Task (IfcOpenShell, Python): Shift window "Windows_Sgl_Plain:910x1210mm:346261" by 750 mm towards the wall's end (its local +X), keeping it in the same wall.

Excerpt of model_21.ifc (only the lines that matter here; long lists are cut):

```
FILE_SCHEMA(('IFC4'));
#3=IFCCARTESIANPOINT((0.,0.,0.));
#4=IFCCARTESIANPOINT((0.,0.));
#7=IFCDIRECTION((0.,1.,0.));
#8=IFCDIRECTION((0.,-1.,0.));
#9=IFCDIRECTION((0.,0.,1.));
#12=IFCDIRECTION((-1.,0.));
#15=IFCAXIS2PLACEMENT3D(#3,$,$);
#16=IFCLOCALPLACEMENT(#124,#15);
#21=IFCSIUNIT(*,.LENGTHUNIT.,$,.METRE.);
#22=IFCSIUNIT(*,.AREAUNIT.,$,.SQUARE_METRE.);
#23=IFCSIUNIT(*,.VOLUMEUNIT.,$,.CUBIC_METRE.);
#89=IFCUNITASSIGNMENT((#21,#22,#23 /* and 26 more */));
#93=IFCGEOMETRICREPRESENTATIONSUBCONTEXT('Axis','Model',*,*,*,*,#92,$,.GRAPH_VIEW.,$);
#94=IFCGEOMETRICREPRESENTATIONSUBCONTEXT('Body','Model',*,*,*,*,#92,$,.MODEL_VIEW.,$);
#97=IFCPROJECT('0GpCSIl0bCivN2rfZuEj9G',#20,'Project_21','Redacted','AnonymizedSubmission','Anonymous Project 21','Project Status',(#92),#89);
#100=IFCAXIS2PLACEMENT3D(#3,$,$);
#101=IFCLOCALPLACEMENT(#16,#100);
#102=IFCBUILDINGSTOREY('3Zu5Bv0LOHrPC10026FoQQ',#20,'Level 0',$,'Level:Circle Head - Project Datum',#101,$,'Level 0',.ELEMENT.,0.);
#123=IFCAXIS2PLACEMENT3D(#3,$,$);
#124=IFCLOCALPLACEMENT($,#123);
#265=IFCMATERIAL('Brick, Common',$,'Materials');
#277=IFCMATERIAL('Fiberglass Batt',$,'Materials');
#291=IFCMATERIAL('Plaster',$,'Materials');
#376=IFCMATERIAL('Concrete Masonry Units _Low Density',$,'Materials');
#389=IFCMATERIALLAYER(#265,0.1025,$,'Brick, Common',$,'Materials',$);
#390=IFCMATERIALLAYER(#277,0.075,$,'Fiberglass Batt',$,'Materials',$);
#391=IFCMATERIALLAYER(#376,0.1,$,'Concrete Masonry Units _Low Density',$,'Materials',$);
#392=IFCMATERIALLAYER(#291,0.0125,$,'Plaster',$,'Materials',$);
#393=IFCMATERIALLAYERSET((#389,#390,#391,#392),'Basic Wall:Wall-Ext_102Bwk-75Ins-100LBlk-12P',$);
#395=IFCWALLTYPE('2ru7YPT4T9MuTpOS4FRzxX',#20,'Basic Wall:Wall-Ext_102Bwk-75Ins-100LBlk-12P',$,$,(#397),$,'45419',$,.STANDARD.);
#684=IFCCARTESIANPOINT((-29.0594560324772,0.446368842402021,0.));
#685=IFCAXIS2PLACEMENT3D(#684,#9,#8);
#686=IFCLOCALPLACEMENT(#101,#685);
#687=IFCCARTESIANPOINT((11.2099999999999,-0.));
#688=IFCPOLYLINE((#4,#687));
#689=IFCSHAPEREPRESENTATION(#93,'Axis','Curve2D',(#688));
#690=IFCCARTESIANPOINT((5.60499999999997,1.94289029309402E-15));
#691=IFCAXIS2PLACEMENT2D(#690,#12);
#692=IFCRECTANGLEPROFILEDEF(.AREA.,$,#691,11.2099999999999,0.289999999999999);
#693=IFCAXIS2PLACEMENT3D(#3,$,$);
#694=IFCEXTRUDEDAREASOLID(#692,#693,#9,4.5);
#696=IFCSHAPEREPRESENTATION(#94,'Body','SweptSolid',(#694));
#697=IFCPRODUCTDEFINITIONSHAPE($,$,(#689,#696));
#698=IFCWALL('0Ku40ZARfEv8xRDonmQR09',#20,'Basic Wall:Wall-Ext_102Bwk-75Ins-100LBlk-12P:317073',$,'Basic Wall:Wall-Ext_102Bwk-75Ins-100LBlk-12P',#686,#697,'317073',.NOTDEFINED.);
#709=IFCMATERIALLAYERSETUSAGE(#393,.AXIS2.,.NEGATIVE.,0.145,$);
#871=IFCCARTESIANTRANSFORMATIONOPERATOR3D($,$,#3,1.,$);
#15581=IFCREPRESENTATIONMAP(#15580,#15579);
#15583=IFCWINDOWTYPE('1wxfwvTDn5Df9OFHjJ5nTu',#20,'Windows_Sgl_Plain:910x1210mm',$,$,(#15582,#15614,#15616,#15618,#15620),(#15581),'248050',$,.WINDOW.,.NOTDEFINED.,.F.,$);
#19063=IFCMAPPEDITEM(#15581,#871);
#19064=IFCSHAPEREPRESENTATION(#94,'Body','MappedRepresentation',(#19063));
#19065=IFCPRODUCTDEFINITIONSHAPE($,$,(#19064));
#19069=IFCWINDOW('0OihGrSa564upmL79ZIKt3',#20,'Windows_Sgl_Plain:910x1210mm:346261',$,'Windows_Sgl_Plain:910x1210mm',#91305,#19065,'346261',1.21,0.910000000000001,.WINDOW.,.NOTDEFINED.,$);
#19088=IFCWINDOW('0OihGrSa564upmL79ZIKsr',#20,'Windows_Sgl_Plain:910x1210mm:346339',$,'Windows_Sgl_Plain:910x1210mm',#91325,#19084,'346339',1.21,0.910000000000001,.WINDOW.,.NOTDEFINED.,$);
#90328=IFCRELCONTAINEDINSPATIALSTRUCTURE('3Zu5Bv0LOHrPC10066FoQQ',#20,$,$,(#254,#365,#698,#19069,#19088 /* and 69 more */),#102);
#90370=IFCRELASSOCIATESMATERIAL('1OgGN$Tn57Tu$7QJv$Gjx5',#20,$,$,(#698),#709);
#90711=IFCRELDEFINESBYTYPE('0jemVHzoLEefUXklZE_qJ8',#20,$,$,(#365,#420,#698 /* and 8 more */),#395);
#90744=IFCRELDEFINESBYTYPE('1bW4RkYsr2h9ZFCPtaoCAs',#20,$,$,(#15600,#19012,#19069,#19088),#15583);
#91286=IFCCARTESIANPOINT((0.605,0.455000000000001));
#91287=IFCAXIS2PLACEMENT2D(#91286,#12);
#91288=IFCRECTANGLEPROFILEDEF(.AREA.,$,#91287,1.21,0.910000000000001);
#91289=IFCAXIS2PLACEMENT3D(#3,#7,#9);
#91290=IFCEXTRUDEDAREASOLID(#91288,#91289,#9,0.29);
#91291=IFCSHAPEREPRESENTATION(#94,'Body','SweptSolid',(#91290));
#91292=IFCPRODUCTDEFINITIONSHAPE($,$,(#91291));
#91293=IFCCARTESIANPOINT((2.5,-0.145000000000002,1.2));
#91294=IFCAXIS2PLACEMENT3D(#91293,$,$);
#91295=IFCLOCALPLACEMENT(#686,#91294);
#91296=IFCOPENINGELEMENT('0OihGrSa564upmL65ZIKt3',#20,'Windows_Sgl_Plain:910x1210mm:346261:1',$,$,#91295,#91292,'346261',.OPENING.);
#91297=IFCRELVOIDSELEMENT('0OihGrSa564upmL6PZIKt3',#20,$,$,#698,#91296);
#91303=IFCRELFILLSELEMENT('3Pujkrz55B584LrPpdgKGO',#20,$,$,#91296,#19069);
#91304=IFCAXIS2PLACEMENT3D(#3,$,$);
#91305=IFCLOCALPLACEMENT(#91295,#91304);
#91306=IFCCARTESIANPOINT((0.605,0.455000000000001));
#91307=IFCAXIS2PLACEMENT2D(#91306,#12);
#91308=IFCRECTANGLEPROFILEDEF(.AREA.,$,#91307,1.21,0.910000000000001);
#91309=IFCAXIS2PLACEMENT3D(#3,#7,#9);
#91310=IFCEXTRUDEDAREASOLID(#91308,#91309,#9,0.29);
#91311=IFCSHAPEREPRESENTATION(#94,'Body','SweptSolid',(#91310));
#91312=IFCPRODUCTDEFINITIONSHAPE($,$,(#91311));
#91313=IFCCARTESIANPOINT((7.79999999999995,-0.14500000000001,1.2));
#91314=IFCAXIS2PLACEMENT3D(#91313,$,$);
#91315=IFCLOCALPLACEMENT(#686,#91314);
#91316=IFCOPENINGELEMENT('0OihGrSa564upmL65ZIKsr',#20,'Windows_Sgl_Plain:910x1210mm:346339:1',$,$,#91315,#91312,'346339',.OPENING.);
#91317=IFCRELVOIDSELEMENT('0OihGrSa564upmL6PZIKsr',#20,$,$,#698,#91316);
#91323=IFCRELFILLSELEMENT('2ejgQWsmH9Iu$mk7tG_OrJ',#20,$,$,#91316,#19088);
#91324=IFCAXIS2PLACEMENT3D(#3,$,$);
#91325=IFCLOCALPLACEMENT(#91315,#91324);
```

```python
import ifcopenshell
import ifcopenshell.api.geometry
import ifcopenshell.util.placement

model = ifcopenshell.open("model_21.ifc")

window = model.by_guid("0OihGrSa564upmL79ZIKt3")
opening = window.FillsVoids[0].RelatingOpeningElement
wall = opening.VoidsElements[0].RelatingBuildingElement

wall_matrix = ifcopenshell.util.placement.get_local_placement(wall.ObjectPlacement)
shift = wall_matrix[:3, 0] * 0.75
before = ifcopenshell.util.placement.get_local_placement(window.ObjectPlacement)[:3, 3].copy()

# The window is placed relative to its opening, so it follows when the opening moves.
matrix = ifcopenshell.util.placement.get_local_placement(opening.ObjectPlacement)
matrix[:3, 3] += shift
ifcopenshell.api.geometry.edit_object_placement(
    model, product=opening, matrix=matrix, is_si=False, should_transform_children=True
)

after = ifcopenshell.util.placement.get_local_placement(window.ObjectPlacement)[:3, 3]
print("window moved by", (after - before).round(3) + 0.0)

model.write("model_21_updated.ifc")
```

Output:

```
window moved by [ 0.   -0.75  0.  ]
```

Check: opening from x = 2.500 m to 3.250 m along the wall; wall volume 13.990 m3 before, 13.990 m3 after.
